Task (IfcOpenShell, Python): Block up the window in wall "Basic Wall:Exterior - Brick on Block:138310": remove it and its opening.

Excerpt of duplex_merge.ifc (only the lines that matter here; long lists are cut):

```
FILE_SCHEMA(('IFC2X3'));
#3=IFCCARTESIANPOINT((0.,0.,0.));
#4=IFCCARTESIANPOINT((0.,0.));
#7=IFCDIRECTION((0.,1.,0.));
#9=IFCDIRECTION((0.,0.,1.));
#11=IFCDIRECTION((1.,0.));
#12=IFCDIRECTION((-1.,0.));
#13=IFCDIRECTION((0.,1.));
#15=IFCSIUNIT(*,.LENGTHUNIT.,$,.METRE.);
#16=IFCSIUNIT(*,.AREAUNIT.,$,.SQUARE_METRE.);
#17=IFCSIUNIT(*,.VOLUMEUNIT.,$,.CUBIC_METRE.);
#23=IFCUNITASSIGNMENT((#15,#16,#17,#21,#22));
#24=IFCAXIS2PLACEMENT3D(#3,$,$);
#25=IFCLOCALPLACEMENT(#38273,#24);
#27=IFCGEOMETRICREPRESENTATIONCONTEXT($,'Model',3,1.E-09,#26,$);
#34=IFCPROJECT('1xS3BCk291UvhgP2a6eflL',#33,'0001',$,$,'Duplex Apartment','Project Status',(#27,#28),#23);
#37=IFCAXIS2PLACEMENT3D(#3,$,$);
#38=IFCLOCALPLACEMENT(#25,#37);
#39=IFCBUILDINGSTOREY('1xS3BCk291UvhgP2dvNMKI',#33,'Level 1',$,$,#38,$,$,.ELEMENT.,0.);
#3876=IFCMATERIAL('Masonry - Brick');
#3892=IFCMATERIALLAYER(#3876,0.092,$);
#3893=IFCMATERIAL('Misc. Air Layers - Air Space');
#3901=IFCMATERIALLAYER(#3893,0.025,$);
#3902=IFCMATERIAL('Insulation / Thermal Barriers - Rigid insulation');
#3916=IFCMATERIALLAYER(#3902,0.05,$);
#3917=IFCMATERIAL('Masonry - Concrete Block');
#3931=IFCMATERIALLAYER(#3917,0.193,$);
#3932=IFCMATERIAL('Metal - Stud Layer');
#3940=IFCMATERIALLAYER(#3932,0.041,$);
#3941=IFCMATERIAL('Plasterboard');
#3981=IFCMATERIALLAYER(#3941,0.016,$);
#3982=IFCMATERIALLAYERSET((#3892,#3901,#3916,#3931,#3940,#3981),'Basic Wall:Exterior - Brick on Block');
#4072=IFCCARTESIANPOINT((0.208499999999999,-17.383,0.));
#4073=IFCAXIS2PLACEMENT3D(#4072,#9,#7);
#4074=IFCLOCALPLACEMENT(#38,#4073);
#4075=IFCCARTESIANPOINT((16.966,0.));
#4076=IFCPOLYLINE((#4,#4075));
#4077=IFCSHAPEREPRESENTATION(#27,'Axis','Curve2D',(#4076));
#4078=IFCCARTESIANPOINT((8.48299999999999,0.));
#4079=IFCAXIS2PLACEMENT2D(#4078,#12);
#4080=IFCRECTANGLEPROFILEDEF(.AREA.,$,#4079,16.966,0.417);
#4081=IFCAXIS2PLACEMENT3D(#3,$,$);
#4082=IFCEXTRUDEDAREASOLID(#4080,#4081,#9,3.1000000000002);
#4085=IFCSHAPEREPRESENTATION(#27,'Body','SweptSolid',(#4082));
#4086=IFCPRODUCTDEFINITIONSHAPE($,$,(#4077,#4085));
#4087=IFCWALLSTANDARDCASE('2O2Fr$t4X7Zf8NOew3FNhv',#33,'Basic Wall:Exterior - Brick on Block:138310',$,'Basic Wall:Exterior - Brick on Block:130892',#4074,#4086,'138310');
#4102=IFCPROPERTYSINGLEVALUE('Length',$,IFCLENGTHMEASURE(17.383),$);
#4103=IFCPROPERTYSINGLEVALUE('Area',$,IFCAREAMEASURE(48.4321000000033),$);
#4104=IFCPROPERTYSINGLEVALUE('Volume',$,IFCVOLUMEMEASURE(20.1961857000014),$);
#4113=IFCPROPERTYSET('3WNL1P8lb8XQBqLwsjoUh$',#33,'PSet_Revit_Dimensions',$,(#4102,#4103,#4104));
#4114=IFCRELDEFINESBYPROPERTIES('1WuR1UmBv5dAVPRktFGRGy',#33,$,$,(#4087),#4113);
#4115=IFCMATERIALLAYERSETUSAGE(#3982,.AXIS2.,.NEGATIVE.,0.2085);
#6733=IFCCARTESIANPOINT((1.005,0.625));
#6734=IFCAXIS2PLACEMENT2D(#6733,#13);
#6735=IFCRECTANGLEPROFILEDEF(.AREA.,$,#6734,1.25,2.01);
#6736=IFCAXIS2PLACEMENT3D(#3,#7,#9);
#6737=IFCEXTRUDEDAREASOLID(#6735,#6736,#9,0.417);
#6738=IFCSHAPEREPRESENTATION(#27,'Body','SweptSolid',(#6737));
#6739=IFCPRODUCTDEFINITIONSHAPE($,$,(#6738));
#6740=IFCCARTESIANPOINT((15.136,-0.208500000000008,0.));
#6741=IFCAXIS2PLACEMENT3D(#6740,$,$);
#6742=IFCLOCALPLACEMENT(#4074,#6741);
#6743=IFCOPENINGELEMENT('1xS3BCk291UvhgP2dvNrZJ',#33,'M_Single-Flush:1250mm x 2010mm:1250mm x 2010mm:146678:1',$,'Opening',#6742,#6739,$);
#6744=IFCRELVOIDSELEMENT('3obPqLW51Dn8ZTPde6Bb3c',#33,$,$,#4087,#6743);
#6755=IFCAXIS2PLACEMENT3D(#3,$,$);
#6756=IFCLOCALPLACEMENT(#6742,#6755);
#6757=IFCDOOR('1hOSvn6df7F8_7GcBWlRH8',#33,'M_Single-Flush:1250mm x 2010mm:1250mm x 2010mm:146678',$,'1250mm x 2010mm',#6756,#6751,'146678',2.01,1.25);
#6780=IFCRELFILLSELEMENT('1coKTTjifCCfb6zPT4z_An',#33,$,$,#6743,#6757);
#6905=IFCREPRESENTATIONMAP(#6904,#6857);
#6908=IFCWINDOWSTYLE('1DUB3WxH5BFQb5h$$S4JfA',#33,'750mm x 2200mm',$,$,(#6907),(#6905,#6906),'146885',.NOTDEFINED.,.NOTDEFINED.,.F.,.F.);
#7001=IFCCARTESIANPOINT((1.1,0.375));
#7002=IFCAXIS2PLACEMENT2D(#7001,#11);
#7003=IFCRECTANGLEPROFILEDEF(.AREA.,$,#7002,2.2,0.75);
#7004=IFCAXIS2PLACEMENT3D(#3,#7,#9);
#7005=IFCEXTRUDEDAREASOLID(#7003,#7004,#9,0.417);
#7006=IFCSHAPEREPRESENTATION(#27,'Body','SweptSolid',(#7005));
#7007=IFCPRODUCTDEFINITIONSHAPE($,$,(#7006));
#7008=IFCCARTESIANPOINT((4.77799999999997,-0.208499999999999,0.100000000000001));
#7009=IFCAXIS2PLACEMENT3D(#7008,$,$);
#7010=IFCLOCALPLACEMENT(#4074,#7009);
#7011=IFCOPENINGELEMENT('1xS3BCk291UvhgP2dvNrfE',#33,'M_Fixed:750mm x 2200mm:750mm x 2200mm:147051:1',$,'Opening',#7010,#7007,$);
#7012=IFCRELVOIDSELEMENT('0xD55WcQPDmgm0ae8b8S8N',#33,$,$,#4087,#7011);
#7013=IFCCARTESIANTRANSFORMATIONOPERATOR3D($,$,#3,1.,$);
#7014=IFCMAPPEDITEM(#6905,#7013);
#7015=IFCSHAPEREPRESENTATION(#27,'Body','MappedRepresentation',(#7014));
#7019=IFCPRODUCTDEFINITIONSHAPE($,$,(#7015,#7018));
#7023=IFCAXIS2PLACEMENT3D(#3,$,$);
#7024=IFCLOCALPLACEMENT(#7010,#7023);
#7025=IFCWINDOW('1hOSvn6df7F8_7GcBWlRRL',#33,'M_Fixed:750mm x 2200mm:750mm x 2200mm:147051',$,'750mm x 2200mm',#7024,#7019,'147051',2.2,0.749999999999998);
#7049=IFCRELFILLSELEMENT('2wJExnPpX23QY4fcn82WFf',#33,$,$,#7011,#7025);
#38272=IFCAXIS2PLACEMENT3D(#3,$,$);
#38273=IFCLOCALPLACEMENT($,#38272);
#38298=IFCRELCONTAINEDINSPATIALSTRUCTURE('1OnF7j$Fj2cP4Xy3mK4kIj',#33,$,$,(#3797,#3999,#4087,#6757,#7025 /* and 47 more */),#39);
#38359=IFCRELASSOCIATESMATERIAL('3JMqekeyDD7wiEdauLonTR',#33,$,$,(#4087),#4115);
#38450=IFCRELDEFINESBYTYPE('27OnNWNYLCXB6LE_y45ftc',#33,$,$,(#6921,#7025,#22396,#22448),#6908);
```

```python
import ifcopenshell
import ifcopenshell.api.feature
import ifcopenshell.api.pset
import ifcopenshell.api.root
import ifcopenshell.geom
import ifcopenshell.util.element
import ifcopenshell.util.shape
import ifcopenshell.util.unit

model = ifcopenshell.open("duplex_merge.ifc")
area_scale = ifcopenshell.util.unit.calculate_unit_scale(model, "AREAUNIT")
volume_scale = ifcopenshell.util.unit.calculate_unit_scale(model, "VOLUMEUNIT")
settings = ifcopenshell.geom.settings()


def volume(element):
    """Net volume in cubic metres, openings subtracted."""
    shape = ifcopenshell.geom.create_shape(settings, element)
    return ifcopenshell.util.shape.get_volume(shape.geometry)


window = model.by_guid("1hOSvn6df7F8_7GcBWlRRL")
opening = window.FillsVoids[0].RelatingOpeningElement
wall = opening.VoidsElements[0].RelatingBuildingElement
before = volume(wall)

ifcopenshell.api.root.remove_product(model, product=window)
ifcopenshell.api.feature.remove_feature(model, feature=opening)

after = volume(wall)
thickness = 0.417  # wall thickness in metres

# Update the wall's stored quantities.
pset = model.by_id(ifcopenshell.util.element.get_pset(wall, "PSet_Revit_Dimensions", should_inherit=False)["id"])
ifcopenshell.api.pset.edit_pset(model, pset=pset, properties={
    "Area": model.create_entity("IfcAreaMeasure", after / thickness / area_scale),
    "Volume": model.create_entity("IfcVolumeMeasure", after / volume_scale),
})

print(f"wall volume {before:.3f} -> {after:.3f} m3")

model.write("duplex_merge_edited.ifc")
```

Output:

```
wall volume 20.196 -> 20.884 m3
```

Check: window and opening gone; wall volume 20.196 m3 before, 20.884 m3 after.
